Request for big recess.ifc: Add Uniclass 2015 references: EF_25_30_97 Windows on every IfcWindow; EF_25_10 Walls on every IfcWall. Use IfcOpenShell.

First a look at what the model holds.

```python
import ifcopenshell

model = ifcopenshell.open("big recess.ifc")
print(model.schema)
print("classifications:", [c.Name for c in model.by_type("IfcClassification")])
for ifc_class in ("IfcDoor", "IfcRoof", "IfcStair", "IfcWall", "IfcWindow"):
    print(ifc_class, len(model.by_type(ifc_class)))
```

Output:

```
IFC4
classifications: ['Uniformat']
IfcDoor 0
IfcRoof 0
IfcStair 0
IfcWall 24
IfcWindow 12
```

```python
import ifcopenshell
import ifcopenshell.api.classification

model = ifcopenshell.open("big recess.ifc")

system = ifcopenshell.api.classification.add_classification(model, classification="Uniclass 2015")

codes = {
    "IfcWindow": ("EF_25_30_97", "Windows"),
    "IfcWall": ("EF_25_10", "Walls"),
}
for ifc_class, (code, name) in codes.items():
    products = model.by_type(ifc_class)
    ifcopenshell.api.classification.add_reference(
        model, products=products, classification=system, identification=code, name=name
    )
    print(code, len(products))

model.write("big recess_updated.ifc")
```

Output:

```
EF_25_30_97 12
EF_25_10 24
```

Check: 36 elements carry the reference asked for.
